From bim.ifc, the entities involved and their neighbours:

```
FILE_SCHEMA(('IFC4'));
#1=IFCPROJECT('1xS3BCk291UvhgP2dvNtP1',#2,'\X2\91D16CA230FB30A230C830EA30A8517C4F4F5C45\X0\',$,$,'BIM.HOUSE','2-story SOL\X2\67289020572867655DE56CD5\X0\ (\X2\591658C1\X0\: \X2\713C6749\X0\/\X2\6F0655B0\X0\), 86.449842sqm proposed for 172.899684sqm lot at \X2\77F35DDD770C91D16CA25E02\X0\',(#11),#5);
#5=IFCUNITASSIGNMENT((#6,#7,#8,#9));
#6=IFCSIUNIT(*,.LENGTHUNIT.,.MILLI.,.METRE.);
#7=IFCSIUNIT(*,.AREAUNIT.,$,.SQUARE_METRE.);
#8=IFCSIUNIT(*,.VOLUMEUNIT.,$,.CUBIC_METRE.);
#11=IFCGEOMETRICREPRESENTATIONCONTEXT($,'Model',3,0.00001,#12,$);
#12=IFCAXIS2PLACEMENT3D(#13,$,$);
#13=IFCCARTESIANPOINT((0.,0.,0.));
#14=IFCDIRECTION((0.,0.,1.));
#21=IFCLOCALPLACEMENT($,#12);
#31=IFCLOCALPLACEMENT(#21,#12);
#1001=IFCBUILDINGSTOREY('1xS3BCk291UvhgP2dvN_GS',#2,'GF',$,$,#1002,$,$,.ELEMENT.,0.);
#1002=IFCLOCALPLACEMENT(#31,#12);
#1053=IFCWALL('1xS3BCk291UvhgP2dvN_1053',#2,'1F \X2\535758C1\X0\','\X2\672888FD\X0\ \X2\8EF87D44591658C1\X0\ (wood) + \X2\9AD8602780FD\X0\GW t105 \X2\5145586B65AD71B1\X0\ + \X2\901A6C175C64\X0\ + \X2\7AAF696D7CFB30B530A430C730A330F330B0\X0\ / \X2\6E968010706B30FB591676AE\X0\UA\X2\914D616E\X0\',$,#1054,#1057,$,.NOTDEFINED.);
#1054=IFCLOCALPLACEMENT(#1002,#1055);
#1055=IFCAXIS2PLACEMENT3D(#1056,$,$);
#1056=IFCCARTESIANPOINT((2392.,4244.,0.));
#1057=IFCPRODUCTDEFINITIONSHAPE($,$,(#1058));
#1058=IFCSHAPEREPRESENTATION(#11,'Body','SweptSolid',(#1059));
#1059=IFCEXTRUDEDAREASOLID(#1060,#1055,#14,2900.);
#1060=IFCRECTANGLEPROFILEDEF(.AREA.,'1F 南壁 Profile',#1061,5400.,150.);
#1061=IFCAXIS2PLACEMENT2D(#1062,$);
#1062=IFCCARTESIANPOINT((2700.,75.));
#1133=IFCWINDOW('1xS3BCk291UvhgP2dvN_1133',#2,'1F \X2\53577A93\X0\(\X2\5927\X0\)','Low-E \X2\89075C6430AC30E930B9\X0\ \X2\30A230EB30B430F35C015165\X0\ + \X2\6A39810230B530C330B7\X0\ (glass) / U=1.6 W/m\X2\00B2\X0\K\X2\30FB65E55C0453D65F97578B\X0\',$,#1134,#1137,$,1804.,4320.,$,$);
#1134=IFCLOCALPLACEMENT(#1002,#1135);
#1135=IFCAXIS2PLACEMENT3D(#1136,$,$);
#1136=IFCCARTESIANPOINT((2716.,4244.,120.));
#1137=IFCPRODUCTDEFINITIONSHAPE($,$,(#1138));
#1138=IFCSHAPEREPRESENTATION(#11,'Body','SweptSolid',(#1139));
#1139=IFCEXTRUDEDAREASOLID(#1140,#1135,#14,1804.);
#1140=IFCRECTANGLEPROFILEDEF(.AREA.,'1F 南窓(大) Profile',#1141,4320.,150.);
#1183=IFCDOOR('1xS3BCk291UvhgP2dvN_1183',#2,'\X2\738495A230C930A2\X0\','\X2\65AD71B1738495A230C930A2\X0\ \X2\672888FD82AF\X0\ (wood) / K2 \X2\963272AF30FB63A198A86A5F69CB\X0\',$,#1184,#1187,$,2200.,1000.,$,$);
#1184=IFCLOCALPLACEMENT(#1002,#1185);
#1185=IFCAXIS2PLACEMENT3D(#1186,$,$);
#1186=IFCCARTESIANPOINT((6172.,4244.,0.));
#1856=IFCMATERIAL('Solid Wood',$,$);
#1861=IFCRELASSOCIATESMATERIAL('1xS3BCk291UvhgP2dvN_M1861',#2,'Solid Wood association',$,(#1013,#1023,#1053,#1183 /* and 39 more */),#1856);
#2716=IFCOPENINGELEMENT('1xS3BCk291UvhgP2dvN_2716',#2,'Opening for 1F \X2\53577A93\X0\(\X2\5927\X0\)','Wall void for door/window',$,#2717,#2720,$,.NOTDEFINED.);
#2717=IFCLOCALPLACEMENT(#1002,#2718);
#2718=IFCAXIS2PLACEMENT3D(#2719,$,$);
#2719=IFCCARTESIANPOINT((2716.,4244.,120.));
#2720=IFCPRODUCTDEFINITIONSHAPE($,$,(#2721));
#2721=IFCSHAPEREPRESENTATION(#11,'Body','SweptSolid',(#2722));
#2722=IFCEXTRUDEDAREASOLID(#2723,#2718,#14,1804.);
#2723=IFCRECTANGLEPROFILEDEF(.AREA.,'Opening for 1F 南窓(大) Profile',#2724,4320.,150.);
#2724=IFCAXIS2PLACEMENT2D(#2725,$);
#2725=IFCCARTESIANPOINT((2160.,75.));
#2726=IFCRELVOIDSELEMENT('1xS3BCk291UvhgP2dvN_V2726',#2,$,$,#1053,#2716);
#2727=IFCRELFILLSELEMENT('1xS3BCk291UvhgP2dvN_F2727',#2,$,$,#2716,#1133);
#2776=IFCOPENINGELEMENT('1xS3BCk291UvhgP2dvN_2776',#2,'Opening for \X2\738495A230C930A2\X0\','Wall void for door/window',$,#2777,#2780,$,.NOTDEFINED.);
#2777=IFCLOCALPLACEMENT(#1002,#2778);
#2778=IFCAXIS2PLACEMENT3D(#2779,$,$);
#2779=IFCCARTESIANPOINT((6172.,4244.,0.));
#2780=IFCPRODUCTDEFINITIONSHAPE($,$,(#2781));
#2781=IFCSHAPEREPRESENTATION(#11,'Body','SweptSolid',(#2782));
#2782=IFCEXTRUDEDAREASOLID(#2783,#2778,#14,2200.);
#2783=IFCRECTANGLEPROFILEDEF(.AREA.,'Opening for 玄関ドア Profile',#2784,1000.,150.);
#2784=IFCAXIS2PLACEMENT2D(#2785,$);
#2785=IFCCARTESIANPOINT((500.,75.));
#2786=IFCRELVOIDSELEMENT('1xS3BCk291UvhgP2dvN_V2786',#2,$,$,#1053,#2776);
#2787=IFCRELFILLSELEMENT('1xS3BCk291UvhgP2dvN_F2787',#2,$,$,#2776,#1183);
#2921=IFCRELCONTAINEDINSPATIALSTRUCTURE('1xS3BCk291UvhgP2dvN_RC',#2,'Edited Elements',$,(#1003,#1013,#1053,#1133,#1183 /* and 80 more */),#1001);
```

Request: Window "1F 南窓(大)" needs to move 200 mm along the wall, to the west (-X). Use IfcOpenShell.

```python
import ifcopenshell
import ifcopenshell.api.geometry
import ifcopenshell.util.placement
import ifcopenshell.util.unit

model = ifcopenshell.open("bim.ifc")
unit_scale = ifcopenshell.util.unit.calculate_unit_scale(model)

window = model.by_guid("1xS3BCk291UvhgP2dvN_1133")
opening = window.FillsVoids[0].RelatingOpeningElement
wall = opening.VoidsElements[0].RelatingBuildingElement

wall_matrix = ifcopenshell.util.placement.get_local_placement(wall.ObjectPlacement)
shift = wall_matrix[:3, 0] * -0.2 / unit_scale
before = ifcopenshell.util.placement.get_local_placement(window.ObjectPlacement)[:3, 3].copy()

# The window is not placed relative to its opening, so move both.
for product in (opening, window):
    matrix = ifcopenshell.util.placement.get_local_placement(product.ObjectPlacement)
    matrix[:3, 3] += shift
    ifcopenshell.api.geometry.edit_object_placement(model, product=product, matrix=matrix, is_si=False)

after = ifcopenshell.util.placement.get_local_placement(window.ObjectPlacement)[:3, 3]
print("window moved by", (after - before).round(3) + 0.0)

model.write("bim_updated.ifc")
```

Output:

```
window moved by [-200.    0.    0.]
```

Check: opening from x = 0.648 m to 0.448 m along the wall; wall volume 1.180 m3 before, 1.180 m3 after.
